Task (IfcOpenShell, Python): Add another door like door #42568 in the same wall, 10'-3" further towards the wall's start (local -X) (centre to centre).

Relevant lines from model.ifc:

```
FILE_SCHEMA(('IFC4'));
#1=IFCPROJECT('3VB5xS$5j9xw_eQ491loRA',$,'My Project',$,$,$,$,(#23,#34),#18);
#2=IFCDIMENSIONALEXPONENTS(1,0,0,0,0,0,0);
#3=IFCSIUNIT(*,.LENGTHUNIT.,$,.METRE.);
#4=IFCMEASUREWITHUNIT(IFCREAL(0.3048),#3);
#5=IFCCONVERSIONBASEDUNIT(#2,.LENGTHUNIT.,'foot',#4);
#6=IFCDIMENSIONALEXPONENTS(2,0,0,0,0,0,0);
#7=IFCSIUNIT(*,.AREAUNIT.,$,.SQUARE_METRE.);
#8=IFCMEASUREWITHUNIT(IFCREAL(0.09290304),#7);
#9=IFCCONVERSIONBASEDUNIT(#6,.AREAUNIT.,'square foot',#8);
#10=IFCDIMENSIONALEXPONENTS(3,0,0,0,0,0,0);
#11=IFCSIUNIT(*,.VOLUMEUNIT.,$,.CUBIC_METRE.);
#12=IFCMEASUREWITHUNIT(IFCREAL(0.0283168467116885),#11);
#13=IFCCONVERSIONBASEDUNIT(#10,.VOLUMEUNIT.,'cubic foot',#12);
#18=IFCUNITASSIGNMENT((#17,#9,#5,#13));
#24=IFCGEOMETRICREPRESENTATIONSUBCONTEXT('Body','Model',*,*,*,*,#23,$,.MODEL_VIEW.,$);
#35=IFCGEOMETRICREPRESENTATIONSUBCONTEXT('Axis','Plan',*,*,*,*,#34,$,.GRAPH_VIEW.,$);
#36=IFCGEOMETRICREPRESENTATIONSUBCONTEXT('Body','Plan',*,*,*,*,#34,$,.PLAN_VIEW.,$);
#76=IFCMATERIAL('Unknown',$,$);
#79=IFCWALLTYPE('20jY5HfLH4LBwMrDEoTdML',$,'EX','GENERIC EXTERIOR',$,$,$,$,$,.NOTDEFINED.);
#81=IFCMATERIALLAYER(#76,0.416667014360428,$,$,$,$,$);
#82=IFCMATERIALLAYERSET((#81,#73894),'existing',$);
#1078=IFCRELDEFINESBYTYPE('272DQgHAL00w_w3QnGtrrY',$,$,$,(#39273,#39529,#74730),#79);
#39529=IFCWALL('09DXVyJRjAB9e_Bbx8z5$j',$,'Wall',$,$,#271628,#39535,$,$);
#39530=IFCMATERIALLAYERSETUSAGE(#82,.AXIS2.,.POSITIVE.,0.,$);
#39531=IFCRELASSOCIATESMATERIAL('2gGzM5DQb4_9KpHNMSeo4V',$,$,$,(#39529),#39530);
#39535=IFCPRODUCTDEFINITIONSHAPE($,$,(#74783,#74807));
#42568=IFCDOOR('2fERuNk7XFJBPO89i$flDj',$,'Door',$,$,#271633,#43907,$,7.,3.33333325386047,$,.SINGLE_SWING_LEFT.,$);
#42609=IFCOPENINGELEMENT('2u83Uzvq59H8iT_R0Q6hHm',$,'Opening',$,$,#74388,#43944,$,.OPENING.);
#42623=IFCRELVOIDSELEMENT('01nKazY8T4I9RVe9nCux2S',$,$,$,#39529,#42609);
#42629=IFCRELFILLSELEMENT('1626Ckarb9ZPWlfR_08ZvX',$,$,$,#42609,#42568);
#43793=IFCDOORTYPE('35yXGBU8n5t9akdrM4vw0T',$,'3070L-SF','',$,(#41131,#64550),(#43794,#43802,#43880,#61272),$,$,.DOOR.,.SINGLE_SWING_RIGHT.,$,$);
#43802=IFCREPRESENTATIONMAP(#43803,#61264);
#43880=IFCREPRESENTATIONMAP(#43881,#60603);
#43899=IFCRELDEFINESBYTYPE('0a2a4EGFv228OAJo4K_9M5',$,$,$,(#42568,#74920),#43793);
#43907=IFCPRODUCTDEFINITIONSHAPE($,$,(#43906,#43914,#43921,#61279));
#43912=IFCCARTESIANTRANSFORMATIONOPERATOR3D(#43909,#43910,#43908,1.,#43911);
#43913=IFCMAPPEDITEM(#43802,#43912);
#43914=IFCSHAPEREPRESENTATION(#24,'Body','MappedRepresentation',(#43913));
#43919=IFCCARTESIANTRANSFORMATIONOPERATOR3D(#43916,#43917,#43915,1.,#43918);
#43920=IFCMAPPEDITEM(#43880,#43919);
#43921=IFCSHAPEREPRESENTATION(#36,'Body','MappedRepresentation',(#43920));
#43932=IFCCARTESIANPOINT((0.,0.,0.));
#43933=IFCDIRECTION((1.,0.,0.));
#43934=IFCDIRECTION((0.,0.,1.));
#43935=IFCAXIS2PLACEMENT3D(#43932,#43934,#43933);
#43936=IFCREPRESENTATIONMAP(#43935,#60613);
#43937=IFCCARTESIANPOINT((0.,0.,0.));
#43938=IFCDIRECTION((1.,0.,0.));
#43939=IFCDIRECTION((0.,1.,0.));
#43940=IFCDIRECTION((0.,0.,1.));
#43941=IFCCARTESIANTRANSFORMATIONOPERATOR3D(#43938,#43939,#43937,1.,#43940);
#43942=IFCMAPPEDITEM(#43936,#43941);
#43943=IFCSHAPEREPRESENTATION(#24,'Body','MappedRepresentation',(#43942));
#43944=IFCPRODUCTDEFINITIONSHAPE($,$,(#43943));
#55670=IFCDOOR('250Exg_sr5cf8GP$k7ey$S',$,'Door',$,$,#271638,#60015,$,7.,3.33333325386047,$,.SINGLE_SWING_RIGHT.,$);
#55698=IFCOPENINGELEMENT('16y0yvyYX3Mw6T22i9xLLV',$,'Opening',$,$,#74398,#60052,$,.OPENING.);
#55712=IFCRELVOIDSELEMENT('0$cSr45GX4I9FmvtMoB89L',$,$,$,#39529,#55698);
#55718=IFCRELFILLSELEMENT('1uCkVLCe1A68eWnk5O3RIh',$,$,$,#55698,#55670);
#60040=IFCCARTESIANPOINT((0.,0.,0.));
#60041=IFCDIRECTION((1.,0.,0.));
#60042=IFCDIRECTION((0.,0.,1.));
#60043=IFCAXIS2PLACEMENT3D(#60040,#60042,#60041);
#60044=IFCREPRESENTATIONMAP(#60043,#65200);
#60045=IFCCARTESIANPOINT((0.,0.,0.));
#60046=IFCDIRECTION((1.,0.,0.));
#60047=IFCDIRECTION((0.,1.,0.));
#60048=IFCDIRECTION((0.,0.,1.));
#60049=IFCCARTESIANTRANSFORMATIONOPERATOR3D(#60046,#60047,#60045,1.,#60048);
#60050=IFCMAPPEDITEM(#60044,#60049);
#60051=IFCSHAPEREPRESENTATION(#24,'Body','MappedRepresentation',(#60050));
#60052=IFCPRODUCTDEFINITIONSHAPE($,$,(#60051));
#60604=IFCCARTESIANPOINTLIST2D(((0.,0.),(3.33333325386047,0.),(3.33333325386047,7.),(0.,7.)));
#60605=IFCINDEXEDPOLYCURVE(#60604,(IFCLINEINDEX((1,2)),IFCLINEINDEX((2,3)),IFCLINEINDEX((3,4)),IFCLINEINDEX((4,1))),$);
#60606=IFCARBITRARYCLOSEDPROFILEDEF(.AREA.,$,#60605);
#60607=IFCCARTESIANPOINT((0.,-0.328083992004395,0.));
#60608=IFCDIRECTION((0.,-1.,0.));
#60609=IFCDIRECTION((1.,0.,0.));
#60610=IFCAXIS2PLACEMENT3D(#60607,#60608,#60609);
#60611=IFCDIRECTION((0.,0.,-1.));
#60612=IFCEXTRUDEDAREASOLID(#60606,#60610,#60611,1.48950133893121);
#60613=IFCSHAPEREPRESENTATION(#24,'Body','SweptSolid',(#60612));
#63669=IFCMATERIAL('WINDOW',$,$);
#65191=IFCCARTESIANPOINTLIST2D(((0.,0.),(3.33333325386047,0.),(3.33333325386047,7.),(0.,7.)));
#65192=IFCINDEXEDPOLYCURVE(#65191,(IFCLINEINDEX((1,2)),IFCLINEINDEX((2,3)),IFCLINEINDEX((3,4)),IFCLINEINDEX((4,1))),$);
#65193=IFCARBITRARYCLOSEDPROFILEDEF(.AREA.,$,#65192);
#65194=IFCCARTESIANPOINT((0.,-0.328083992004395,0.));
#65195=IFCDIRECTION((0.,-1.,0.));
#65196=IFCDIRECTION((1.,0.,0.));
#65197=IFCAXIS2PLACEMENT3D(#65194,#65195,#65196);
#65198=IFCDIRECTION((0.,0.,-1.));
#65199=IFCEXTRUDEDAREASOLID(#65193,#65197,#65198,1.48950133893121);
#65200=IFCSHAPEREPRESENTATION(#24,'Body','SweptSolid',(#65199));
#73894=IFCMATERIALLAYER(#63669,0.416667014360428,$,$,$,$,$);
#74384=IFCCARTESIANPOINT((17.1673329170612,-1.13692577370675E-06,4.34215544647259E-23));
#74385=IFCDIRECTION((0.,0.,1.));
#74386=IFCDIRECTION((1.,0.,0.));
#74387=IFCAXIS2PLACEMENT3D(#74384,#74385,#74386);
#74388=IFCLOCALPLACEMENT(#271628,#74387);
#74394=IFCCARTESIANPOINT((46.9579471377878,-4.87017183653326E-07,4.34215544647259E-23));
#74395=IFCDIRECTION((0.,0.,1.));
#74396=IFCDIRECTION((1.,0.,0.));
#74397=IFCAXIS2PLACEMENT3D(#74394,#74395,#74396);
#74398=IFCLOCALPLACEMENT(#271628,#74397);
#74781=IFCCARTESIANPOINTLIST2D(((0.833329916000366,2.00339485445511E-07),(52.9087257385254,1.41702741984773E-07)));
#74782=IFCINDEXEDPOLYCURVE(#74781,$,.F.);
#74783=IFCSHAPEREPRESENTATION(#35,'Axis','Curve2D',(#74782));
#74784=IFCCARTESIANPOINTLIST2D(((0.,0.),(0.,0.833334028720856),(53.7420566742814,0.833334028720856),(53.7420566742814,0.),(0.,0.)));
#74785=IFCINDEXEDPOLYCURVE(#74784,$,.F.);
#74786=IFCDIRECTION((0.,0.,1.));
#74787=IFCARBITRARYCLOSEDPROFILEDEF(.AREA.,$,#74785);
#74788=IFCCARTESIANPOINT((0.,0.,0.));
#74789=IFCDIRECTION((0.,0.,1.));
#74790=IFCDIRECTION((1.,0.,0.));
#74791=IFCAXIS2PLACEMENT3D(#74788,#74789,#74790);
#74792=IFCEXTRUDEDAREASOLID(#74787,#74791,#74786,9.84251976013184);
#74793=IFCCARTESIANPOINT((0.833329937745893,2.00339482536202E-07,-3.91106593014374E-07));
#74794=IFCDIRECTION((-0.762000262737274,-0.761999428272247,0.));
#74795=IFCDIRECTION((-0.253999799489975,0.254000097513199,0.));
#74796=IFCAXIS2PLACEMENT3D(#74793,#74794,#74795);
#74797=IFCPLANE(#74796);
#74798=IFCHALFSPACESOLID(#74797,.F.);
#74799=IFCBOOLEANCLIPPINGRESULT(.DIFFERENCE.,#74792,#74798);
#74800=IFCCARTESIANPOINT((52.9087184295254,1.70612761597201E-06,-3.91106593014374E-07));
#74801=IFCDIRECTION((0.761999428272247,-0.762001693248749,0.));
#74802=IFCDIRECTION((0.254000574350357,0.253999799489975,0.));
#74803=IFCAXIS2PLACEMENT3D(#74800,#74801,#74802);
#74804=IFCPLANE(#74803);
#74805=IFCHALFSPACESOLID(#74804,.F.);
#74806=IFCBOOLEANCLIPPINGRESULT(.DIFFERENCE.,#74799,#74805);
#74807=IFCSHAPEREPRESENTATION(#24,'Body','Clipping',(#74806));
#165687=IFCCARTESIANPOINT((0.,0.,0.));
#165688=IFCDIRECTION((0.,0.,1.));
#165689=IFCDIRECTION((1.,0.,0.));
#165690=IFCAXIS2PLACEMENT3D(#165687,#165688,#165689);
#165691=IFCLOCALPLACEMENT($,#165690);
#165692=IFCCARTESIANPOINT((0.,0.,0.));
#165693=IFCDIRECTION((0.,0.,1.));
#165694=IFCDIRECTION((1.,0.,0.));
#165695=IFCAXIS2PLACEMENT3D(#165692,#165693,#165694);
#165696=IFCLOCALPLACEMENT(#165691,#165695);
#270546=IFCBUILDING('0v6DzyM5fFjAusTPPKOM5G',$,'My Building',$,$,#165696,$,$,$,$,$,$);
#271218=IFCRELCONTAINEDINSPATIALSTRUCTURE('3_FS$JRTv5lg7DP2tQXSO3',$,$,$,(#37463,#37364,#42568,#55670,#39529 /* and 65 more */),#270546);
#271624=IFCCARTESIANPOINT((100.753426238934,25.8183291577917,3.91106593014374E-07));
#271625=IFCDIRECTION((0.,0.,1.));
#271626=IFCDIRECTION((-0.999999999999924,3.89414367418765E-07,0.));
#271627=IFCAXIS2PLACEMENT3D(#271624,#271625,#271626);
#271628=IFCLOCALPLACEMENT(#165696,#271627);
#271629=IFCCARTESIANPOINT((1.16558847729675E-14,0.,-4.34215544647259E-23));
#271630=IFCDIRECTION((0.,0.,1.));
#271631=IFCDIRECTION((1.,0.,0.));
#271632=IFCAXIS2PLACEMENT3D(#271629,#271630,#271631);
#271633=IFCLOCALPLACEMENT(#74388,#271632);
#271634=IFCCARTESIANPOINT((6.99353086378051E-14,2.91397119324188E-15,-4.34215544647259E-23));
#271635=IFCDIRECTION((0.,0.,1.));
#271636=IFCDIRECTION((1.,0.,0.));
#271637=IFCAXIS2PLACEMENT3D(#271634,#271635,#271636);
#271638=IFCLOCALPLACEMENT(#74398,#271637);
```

```python
import ifcopenshell
import ifcopenshell.api.feature
import ifcopenshell.api.geometry
import ifcopenshell.api.root
import ifcopenshell.geom
import ifcopenshell.util.element
import ifcopenshell.util.placement
import ifcopenshell.util.shape
import ifcopenshell.util.unit

model = ifcopenshell.open("model.ifc")
unit_scale = ifcopenshell.util.unit.calculate_unit_scale(model)
settings = ifcopenshell.geom.settings()


def volume(element):
    """Net volume in cubic metres, openings subtracted."""
    shape = ifcopenshell.geom.create_shape(settings, element)
    return ifcopenshell.util.shape.get_volume(shape.geometry)


door = model.by_guid("2fERuNk7XFJBPO89i$flDj")
opening = door.FillsVoids[0].RelatingOpeningElement
wall = opening.VoidsElements[0].RelatingBuildingElement
before = volume(wall)
shift = ifcopenshell.util.placement.get_local_placement(wall.ObjectPlacement)[:3, 0] * -123 * 0.0254 / unit_scale

# copy_class copies the void relationship, type, container and properties, but no geometry.
new_opening = ifcopenshell.api.root.copy_class(model, product=opening)
new_opening.Representation = ifcopenshell.util.element.copy_deep(
    model, opening.Representation, exclude=["IfcGeometricRepresentationContext", "IfcRepresentationMap"]
)
new_door = ifcopenshell.api.root.copy_class(model, product=door)
new_door.Representation = ifcopenshell.util.element.copy_deep(
    model, door.Representation, exclude=["IfcGeometricRepresentationContext", "IfcRepresentationMap"]
)
ifcopenshell.api.feature.add_filling(model, opening=new_opening, element=new_door)

for old, new in ((opening, new_opening), (door, new_door)):
    matrix = ifcopenshell.util.placement.get_local_placement(old.ObjectPlacement)
    matrix[:3, 3] += shift
    ifcopenshell.api.geometry.edit_object_placement(model, product=new, matrix=matrix, is_si=False)

after = volume(wall)

print(f"wall volume {before:.3f} -> {after:.3f} m3")

model.write("model_edited.ifc")
```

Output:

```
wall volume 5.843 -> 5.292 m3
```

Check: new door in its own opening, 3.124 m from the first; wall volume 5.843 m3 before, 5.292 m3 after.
